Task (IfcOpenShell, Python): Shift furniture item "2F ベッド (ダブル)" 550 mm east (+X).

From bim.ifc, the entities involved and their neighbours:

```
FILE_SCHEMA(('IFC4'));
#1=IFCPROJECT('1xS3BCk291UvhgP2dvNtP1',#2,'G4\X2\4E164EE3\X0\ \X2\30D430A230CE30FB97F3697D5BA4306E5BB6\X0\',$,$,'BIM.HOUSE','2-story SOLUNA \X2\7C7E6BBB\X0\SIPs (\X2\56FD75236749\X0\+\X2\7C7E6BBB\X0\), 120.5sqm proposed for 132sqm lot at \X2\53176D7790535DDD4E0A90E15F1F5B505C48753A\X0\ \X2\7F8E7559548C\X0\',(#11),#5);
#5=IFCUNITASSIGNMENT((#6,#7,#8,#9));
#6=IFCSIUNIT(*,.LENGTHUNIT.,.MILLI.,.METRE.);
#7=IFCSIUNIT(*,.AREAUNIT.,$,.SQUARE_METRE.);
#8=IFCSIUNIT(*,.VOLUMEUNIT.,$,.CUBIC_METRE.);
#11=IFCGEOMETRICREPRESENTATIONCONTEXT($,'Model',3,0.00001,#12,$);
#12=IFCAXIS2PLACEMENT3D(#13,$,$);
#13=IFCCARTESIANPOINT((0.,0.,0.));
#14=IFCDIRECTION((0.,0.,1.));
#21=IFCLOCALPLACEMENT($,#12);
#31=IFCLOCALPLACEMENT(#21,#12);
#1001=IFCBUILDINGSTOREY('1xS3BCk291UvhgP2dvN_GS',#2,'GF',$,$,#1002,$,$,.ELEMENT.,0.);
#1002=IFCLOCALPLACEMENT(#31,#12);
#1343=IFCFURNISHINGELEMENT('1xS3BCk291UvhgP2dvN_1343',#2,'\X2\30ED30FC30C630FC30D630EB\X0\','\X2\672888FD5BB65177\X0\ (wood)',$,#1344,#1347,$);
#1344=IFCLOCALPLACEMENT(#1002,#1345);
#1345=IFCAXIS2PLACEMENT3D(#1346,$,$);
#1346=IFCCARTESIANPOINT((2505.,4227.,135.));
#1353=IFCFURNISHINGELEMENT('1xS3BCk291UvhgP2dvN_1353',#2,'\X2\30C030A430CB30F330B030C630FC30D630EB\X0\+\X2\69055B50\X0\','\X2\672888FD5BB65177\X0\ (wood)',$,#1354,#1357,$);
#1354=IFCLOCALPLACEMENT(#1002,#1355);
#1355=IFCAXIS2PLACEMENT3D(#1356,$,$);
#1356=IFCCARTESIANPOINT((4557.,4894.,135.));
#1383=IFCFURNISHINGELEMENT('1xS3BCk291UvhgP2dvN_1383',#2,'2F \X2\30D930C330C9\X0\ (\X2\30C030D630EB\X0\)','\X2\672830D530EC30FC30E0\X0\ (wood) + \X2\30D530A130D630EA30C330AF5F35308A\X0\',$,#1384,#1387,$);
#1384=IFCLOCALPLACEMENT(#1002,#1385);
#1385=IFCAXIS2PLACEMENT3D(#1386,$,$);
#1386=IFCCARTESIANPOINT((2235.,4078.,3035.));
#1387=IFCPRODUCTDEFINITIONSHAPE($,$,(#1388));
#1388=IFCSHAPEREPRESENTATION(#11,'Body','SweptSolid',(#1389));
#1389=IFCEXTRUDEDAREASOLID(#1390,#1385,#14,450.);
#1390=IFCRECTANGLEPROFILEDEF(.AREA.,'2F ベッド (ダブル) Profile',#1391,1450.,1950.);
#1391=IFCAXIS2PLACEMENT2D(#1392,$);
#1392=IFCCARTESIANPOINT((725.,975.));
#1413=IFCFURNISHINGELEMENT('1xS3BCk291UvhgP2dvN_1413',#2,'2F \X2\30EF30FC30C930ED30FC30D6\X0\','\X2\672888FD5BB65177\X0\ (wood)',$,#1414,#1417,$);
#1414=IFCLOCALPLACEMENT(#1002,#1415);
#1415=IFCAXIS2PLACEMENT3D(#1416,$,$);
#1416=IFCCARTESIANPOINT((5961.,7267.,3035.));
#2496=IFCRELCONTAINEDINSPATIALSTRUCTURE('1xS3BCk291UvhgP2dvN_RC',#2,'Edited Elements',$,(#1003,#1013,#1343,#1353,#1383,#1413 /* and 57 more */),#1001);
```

```python
import ifcopenshell
import ifcopenshell.api.geometry
import ifcopenshell.util.placement
import ifcopenshell.util.unit

model = ifcopenshell.open("bim.ifc")
unit_scale = ifcopenshell.util.unit.calculate_unit_scale(model)

item = model.by_guid("1xS3BCk291UvhgP2dvN_1383")
matrix = ifcopenshell.util.placement.get_local_placement(item.ObjectPlacement)
matrix[0, 3] += 0.55 / unit_scale
ifcopenshell.api.geometry.edit_object_placement(model, product=item, matrix=matrix, is_si=False)

print(ifcopenshell.util.placement.get_local_placement(item.ObjectPlacement).round(3) + 0.0)

model.write("bim_v2.ifc")
```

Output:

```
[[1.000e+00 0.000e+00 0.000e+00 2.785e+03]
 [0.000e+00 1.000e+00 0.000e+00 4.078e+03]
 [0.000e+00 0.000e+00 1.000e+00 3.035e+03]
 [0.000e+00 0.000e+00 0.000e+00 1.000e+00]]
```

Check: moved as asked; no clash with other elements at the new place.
